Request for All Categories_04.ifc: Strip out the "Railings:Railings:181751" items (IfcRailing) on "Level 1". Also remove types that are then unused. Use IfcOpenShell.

First a look at what the model holds.

```python
import ifcopenshell
import ifcopenshell.util.element

model = ifcopenshell.open("All Categories_04.ifc")
print(model.schema)
storey = next(s for s in model.by_type("IfcBuildingStorey") if s.Name == "Level 1")
railings = [e for e in ifcopenshell.util.element.get_decomposition(storey) if e.is_a("IfcRailing")]
seen = {}
for e in railings:
    element_type = ifcopenshell.util.element.get_type(e)
    name = element_type.Name if element_type not in (None, e) else None
    seen[name] = seen.get(name, 0) + 1
for name, count in sorted(seen.items(), key=str):
    print(count, "x", name)
```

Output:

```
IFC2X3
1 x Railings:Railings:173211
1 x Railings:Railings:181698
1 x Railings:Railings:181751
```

```python
import ifcopenshell
import ifcopenshell.api.root
import ifcopenshell.util.element

model = ifcopenshell.open("All Categories_04.ifc")

storey = next(s for s in model.by_type("IfcBuildingStorey") if s.Name == "Level 1")
railings = [e for e in ifcopenshell.util.element.get_decomposition(storey) if e.is_a("IfcRailing")]
targets = [e for e in railings if (t := ifcopenshell.util.element.get_type(e)) not in (None, e) and t.Name == "Railings:Railings:181751"]
types = {ifcopenshell.util.element.get_type(e) for e in targets} - {None, *targets}

for e in targets:
    ifcopenshell.api.root.remove_product(model, product=e)
print(len(targets), "removed")

unused = [t for t in types if not ifcopenshell.util.element.get_types(t)]
for t in unused:
    ifcopenshell.api.root.remove_product(model, product=t)
print(len(unused), "unused types removed")

model.write("All Categories_04-out.ifc")
```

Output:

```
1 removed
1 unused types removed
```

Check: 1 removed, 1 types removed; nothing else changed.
